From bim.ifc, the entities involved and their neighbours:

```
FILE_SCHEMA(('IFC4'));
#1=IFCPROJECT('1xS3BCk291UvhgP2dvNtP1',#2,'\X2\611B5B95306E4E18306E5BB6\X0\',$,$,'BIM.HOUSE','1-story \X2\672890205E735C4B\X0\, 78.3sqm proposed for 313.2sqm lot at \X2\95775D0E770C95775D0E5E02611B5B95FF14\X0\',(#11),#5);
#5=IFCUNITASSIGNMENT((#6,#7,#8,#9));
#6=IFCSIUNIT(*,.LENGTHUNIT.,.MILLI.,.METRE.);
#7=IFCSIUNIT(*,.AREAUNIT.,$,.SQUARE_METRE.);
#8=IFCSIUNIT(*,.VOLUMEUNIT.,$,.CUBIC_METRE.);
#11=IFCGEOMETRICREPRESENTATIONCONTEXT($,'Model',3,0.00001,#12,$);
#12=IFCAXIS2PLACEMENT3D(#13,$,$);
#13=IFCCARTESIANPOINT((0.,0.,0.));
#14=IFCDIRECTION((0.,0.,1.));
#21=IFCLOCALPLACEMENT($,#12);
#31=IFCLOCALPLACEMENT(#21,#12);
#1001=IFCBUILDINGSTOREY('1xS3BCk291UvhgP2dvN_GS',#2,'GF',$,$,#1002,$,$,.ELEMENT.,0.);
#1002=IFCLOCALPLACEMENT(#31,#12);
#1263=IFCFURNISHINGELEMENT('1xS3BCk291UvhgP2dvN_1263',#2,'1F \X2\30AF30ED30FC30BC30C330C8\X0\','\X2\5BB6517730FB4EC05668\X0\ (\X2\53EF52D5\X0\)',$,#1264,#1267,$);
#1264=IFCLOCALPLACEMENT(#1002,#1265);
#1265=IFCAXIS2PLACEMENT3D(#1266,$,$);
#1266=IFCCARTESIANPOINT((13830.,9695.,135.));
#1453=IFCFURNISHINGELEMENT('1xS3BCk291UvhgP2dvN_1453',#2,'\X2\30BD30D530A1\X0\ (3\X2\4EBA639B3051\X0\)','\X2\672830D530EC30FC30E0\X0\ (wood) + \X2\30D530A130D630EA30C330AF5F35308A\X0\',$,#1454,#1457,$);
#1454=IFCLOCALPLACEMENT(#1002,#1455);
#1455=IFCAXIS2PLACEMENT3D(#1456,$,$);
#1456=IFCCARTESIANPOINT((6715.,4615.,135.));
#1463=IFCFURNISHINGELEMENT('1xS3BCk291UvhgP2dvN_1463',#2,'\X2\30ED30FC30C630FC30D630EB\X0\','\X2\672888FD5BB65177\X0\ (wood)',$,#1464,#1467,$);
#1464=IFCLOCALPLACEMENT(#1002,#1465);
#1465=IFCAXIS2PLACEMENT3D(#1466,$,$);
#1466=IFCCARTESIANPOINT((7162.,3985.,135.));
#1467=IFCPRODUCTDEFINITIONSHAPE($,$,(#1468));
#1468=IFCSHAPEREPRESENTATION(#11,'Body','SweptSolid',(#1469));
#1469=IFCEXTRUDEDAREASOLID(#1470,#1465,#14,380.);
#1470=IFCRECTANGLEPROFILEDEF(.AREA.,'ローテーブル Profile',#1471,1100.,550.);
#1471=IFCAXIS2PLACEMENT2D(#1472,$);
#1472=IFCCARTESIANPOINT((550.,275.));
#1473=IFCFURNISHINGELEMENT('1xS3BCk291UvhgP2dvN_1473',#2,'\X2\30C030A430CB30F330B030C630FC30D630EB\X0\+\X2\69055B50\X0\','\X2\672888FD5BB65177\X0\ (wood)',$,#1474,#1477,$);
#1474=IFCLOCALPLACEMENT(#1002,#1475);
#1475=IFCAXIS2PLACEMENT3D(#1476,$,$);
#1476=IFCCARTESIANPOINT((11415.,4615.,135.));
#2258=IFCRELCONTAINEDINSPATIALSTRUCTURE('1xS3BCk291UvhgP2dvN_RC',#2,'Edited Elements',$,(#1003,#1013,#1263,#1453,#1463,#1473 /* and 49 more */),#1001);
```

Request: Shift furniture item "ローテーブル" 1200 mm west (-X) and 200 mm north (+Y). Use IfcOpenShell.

```python
import ifcopenshell
import ifcopenshell.api.geometry
import ifcopenshell.util.placement
import ifcopenshell.util.unit

model = ifcopenshell.open("bim.ifc")
unit_scale = ifcopenshell.util.unit.calculate_unit_scale(model)

item = model.by_guid("1xS3BCk291UvhgP2dvN_1463")
matrix = ifcopenshell.util.placement.get_local_placement(item.ObjectPlacement)
matrix[0, 3] -= 1.2 / unit_scale
matrix[1, 3] += 0.2 / unit_scale
ifcopenshell.api.geometry.edit_object_placement(model, product=item, matrix=matrix, is_si=False)

print(ifcopenshell.util.placement.get_local_placement(item.ObjectPlacement).round(3) + 0.0)

model.write("bim_edited.ifc")
```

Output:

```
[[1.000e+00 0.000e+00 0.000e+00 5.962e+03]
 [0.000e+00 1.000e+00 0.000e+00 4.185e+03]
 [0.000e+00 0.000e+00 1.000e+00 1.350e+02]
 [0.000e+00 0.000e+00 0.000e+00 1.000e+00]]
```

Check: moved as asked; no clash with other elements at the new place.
